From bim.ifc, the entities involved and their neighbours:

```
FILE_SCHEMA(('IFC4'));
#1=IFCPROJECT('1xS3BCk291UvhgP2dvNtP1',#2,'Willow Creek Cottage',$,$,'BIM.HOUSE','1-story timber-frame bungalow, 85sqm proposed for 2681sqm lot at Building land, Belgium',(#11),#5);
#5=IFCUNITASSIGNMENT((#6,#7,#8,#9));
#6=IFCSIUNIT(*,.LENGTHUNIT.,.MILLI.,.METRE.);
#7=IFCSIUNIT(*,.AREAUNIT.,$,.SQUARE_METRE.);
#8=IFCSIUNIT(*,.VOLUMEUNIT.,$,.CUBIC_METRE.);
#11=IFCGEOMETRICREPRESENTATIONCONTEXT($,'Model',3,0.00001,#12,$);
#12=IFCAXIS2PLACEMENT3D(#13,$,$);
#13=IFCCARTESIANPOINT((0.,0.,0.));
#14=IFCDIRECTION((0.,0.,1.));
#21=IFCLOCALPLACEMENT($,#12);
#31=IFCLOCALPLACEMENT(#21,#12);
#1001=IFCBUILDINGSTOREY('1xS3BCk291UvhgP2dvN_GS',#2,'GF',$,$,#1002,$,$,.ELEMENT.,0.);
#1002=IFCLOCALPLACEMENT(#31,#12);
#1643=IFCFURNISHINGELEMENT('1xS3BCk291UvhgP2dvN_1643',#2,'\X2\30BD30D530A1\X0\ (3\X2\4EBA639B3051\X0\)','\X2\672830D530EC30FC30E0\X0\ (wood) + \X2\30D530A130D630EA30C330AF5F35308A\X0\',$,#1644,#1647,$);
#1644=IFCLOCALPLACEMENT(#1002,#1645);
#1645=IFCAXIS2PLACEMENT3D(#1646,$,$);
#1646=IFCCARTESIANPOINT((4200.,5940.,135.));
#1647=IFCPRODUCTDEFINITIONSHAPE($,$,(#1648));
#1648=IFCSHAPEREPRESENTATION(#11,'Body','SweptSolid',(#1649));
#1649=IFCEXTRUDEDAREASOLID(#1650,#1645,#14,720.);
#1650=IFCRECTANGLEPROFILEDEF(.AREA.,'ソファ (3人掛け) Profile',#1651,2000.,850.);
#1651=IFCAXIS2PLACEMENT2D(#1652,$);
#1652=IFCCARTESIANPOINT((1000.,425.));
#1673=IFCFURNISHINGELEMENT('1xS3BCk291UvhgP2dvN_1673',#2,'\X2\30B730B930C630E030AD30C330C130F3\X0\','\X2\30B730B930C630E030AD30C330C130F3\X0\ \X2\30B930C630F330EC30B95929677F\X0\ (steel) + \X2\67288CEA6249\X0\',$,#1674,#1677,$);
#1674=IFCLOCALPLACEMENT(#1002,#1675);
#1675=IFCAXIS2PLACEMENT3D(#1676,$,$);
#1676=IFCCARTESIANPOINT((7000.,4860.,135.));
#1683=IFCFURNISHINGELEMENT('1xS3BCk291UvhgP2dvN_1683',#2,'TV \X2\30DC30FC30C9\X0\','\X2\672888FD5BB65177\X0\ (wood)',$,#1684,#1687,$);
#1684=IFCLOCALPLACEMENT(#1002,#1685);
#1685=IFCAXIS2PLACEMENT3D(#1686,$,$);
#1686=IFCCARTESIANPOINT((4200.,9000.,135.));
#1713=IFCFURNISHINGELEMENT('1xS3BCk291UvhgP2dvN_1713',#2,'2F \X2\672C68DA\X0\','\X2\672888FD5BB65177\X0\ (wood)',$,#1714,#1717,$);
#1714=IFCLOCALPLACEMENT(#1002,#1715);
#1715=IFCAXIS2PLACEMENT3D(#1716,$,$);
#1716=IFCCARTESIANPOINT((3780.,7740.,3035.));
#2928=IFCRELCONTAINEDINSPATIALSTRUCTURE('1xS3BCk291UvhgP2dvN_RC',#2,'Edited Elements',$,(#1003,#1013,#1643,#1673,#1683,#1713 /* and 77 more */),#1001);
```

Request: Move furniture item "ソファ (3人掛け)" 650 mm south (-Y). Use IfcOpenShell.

```python
import ifcopenshell
import ifcopenshell.api.geometry
import ifcopenshell.util.placement

model = ifcopenshell.open("bim.ifc")

item = model.by_guid("1xS3BCk291UvhgP2dvN_1643")
matrix = ifcopenshell.util.placement.get_local_placement(item.ObjectPlacement)
matrix[1, 3] -= 650.0
ifcopenshell.api.geometry.edit_object_placement(model, product=item, matrix=matrix, is_si=False)

print(ifcopenshell.util.placement.get_local_placement(item.ObjectPlacement).round(3) + 0.0)

model.write("bim_updated.ifc")
```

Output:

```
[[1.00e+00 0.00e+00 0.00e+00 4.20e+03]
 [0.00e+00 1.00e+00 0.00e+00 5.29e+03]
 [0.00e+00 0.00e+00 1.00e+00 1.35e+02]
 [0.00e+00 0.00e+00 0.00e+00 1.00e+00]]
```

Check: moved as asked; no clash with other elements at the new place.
